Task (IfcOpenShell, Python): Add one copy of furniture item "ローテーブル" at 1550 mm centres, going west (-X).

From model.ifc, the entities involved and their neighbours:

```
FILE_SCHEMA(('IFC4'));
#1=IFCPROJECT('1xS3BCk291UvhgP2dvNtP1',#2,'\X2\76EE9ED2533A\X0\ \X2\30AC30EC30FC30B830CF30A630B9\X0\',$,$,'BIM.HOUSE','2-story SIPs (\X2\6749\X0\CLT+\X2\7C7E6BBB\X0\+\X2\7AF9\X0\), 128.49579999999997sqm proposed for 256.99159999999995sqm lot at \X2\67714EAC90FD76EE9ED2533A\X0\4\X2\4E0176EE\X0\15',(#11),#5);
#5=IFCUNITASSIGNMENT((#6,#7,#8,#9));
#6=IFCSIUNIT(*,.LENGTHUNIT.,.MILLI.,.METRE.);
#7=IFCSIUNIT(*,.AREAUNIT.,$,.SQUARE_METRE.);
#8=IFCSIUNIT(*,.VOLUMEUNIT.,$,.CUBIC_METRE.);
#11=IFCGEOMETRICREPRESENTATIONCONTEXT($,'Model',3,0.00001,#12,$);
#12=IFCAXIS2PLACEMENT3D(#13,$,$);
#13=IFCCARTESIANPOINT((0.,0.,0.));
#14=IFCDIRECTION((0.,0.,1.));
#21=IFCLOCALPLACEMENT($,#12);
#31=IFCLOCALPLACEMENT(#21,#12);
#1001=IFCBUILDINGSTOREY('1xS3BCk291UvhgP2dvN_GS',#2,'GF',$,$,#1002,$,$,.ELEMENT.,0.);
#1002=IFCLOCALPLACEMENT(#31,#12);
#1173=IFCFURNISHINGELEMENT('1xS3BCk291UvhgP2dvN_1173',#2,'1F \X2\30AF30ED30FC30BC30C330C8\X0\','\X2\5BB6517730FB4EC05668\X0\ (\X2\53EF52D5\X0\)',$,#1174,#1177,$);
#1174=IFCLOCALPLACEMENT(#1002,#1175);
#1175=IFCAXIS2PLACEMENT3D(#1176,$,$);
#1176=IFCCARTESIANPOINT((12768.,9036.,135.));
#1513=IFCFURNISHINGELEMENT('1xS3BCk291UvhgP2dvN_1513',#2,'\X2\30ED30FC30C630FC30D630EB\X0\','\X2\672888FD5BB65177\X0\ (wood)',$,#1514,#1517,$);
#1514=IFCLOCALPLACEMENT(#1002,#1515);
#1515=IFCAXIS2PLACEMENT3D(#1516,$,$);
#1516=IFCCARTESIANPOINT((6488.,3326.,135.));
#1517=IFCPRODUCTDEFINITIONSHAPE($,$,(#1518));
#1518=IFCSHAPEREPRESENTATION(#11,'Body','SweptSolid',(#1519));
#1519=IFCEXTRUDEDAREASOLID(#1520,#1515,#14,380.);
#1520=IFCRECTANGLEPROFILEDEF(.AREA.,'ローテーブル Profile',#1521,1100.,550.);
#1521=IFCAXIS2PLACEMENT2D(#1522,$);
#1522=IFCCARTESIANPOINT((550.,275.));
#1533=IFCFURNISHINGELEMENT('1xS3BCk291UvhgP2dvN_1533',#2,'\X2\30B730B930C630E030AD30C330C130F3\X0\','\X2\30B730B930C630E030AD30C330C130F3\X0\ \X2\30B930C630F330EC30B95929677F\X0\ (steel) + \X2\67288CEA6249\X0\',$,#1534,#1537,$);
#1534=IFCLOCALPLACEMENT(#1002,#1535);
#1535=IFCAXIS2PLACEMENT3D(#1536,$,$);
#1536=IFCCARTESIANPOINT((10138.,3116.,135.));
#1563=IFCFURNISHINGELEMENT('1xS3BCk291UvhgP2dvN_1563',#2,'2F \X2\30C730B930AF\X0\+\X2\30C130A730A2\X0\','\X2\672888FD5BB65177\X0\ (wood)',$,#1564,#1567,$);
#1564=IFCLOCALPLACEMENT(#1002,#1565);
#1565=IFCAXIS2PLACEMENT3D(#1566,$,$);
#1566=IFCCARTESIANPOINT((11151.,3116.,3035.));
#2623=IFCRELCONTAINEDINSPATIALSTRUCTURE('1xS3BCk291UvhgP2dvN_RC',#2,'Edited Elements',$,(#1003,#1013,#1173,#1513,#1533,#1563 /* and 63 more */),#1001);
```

```python
import numpy as np
import ifcopenshell
import ifcopenshell.api.geometry
import ifcopenshell.api.root
import ifcopenshell.util.element
import ifcopenshell.util.placement

model = ifcopenshell.open("model.ifc")


def reuse_history(source, copy):
    """copy_class also copies each property set's owner history, people and application; keep the originals."""
    for rel in copy.IsDefinedBy:
        if rel.is_a("IfcRelDefinesByProperties") and (history := rel.RelatingPropertyDefinition.OwnerHistory):
            rel.RelatingPropertyDefinition.OwnerHistory = source.OwnerHistory
            ifcopenshell.util.element.remove_deep2(model, history)


source = model.by_id(1513)
base = ifcopenshell.util.placement.get_local_placement(source.ObjectPlacement)
step = np.array([-1.0, 0.0, 0.0]) * 1550.0

for i in range(1, 2):
    copy = ifcopenshell.api.root.copy_class(model, product=source)
    copy.Representation = ifcopenshell.util.element.copy_deep(
        model, source.Representation, exclude=["IfcGeometricRepresentationContext", "IfcRepresentationMap"]
    )
    reuse_history(source, copy)
    matrix = base.copy()
    matrix[:3, 3] += i * step
    print("added at", matrix[:3, 3].round(3) + 0.0)
    ifcopenshell.api.geometry.edit_object_placement(model, product=copy, matrix=matrix, is_si=False)

model.write("model_rev.ifc")
```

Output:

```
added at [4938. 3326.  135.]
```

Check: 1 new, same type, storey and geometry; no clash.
